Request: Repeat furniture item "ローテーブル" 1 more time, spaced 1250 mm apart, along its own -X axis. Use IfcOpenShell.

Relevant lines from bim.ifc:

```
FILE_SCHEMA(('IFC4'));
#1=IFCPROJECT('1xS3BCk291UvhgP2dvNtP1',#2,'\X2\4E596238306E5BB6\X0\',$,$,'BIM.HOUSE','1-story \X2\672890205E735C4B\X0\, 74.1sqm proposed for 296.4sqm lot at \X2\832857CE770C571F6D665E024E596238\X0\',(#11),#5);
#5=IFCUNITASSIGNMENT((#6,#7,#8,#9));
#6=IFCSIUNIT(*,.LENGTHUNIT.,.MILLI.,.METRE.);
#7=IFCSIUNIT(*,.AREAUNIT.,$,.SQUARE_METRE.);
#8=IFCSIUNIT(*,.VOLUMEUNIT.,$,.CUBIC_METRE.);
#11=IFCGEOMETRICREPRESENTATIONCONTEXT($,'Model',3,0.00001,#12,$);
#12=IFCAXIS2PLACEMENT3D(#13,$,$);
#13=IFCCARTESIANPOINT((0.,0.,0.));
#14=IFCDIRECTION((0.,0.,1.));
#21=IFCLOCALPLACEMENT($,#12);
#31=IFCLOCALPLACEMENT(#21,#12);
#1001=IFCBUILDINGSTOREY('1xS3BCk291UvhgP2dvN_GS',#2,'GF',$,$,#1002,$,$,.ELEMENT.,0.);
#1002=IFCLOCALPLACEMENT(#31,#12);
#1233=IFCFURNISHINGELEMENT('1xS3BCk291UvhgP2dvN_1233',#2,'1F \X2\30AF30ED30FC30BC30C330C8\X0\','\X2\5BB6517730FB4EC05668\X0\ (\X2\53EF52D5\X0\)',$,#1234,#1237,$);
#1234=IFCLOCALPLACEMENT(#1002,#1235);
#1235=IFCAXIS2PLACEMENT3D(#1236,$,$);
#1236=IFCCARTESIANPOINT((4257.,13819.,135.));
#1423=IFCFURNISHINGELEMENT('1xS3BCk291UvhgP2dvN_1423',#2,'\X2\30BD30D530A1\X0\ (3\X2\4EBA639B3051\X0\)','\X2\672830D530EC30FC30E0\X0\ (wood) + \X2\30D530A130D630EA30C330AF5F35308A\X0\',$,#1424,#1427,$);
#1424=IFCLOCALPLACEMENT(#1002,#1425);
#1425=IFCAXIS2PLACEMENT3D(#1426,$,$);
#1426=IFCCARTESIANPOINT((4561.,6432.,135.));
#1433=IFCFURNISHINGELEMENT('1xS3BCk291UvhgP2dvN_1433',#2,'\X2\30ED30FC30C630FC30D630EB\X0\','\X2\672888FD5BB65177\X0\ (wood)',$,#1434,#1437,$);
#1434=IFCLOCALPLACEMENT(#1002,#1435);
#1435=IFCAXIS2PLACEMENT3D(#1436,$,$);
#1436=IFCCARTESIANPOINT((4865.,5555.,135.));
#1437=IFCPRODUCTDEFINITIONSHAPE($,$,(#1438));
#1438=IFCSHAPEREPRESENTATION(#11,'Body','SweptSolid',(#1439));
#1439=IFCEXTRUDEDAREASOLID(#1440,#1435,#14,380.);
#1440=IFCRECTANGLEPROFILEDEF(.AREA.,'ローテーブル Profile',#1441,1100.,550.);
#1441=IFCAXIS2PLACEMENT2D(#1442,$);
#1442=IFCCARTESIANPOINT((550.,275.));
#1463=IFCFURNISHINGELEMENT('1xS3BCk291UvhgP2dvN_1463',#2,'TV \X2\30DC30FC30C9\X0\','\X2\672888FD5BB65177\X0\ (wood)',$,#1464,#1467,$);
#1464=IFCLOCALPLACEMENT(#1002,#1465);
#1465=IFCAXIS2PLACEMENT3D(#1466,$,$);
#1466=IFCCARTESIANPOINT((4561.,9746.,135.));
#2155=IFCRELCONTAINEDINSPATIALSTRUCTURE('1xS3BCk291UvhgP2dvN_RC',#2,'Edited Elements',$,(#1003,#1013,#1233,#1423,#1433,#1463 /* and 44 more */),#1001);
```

```python
import ifcopenshell
import ifcopenshell.api.geometry
import ifcopenshell.api.root
import ifcopenshell.util.element
import ifcopenshell.util.placement
import ifcopenshell.util.unit

model = ifcopenshell.open("bim.ifc")
unit_scale = ifcopenshell.util.unit.calculate_unit_scale(model)


def reuse_history(source, copy):
    """copy_class also copies each property set's owner history, people and application; keep the originals."""
    for rel in copy.IsDefinedBy:
        if rel.is_a("IfcRelDefinesByProperties") and (history := rel.RelatingPropertyDefinition.OwnerHistory):
            rel.RelatingPropertyDefinition.OwnerHistory = source.OwnerHistory
            ifcopenshell.util.element.remove_deep2(model, history)


source = model.by_guid("1xS3BCk291UvhgP2dvN_1433")
base = ifcopenshell.util.placement.get_local_placement(source.ObjectPlacement)
step = -base[:3, 0] * 1.25 / unit_scale

for i in range(1, 2):
    copy = ifcopenshell.api.root.copy_class(model, product=source)
    copy.Representation = ifcopenshell.util.element.copy_deep(
        model, source.Representation, exclude=["IfcGeometricRepresentationContext", "IfcRepresentationMap"]
    )
    reuse_history(source, copy)
    matrix = base.copy()
    matrix[:3, 3] += i * step
    print("added at", matrix[:3, 3].round(3) + 0.0)
    ifcopenshell.api.geometry.edit_object_placement(model, product=copy, matrix=matrix, is_si=False)

model.write("bim_edited.ifc")
```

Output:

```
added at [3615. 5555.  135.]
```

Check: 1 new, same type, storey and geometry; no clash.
